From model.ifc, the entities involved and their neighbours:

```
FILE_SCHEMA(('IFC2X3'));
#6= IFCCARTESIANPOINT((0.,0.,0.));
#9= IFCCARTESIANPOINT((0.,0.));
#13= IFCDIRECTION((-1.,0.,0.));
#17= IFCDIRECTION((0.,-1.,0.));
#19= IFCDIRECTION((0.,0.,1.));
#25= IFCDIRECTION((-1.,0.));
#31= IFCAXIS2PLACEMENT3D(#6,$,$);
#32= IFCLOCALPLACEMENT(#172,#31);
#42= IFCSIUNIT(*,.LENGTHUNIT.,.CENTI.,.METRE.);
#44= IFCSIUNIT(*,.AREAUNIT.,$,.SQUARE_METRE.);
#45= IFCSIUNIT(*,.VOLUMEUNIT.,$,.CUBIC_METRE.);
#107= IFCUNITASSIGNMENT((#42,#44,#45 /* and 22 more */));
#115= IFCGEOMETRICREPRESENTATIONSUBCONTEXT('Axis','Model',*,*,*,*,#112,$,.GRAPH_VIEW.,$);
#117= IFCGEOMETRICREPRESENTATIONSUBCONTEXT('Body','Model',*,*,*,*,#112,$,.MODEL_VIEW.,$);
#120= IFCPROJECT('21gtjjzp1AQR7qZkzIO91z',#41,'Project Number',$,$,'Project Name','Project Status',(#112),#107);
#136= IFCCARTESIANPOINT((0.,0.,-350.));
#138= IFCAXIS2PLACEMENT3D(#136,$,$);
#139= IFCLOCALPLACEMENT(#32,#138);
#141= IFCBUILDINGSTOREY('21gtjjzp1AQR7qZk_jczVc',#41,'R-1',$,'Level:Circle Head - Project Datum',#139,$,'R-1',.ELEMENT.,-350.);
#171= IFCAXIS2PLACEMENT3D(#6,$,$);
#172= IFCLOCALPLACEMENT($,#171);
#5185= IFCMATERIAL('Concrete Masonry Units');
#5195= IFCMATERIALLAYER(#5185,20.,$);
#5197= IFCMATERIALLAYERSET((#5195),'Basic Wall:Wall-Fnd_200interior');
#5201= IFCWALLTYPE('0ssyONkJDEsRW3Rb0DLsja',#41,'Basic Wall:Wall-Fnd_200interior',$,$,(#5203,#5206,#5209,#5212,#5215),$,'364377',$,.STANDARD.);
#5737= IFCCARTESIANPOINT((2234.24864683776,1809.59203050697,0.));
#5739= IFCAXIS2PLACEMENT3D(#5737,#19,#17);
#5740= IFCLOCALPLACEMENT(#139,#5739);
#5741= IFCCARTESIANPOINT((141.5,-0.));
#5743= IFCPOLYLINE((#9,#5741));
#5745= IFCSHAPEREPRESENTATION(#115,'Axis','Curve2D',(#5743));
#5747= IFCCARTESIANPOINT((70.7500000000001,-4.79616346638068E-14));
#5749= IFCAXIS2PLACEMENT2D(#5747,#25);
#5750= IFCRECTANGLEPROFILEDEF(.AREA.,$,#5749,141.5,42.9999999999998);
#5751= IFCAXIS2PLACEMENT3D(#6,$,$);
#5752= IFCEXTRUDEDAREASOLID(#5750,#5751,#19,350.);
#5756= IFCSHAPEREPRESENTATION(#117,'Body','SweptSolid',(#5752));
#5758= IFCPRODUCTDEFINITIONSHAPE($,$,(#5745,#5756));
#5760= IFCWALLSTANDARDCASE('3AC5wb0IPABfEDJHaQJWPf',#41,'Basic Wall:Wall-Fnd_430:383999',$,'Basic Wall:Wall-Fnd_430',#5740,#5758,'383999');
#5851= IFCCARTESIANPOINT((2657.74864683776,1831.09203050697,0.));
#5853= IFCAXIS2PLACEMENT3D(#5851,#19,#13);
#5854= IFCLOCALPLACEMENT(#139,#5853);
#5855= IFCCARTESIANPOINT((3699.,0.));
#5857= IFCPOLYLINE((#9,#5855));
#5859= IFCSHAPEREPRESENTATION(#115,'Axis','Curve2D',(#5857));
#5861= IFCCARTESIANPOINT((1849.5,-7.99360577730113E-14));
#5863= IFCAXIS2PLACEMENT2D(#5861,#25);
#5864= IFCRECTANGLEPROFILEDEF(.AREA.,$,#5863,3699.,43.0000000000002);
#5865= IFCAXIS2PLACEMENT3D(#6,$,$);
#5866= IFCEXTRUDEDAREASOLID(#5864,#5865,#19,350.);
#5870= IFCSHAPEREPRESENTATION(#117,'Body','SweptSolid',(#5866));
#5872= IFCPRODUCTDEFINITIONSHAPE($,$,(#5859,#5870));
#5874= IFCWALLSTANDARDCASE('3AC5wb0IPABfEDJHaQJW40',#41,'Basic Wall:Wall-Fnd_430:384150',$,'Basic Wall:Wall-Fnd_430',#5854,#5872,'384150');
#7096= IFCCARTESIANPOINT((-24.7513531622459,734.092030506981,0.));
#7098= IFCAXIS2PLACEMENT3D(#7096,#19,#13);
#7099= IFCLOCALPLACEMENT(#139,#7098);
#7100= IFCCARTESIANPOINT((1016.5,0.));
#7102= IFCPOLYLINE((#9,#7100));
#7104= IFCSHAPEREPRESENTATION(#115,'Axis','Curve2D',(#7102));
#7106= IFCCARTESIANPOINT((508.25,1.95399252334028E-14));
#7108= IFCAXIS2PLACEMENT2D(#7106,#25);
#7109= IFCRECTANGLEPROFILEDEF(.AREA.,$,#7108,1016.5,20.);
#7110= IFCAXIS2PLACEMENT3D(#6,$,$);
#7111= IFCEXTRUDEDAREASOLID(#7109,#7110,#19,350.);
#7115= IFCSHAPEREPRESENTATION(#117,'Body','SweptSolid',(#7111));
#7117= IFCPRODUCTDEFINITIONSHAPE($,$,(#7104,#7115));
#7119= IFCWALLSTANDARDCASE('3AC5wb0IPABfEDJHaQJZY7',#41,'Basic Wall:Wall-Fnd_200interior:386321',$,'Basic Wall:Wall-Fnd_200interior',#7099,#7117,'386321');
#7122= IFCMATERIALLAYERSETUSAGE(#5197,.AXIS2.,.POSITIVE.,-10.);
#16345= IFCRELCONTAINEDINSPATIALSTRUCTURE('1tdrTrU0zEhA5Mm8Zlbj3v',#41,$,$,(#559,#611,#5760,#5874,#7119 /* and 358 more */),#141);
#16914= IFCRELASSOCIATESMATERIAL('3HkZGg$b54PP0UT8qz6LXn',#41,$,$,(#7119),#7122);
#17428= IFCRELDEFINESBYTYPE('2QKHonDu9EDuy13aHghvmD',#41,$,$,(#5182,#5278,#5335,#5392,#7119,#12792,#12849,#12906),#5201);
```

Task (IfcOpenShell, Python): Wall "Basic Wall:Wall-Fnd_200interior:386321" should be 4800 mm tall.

```python
import ifcopenshell
import ifcopenshell.geom
import ifcopenshell.util.representation
import ifcopenshell.util.shape
import ifcopenshell.util.unit

model = ifcopenshell.open("model.ifc")
unit_scale = ifcopenshell.util.unit.calculate_unit_scale(model)
settings = ifcopenshell.geom.settings()


def volume(element):
    """Net volume in cubic metres, openings subtracted."""
    shape = ifcopenshell.geom.create_shape(settings, element)
    return ifcopenshell.util.shape.get_volume(shape.geometry)


wall = model.by_id(7119)
before = volume(wall)

body = ifcopenshell.util.representation.get_representation(wall, "Model", "Body")
solid = body.Items[0]
old_height = solid.Depth
solid.Depth = 4.8 / unit_scale
after = volume(wall)

print(f"height {old_height:g} -> {solid.Depth:g}, volume {before:.3f} -> {after:.3f} m3")

model.write("model_updated.ifc")
```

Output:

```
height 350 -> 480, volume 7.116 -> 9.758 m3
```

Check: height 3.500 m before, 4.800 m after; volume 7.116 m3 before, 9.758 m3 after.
